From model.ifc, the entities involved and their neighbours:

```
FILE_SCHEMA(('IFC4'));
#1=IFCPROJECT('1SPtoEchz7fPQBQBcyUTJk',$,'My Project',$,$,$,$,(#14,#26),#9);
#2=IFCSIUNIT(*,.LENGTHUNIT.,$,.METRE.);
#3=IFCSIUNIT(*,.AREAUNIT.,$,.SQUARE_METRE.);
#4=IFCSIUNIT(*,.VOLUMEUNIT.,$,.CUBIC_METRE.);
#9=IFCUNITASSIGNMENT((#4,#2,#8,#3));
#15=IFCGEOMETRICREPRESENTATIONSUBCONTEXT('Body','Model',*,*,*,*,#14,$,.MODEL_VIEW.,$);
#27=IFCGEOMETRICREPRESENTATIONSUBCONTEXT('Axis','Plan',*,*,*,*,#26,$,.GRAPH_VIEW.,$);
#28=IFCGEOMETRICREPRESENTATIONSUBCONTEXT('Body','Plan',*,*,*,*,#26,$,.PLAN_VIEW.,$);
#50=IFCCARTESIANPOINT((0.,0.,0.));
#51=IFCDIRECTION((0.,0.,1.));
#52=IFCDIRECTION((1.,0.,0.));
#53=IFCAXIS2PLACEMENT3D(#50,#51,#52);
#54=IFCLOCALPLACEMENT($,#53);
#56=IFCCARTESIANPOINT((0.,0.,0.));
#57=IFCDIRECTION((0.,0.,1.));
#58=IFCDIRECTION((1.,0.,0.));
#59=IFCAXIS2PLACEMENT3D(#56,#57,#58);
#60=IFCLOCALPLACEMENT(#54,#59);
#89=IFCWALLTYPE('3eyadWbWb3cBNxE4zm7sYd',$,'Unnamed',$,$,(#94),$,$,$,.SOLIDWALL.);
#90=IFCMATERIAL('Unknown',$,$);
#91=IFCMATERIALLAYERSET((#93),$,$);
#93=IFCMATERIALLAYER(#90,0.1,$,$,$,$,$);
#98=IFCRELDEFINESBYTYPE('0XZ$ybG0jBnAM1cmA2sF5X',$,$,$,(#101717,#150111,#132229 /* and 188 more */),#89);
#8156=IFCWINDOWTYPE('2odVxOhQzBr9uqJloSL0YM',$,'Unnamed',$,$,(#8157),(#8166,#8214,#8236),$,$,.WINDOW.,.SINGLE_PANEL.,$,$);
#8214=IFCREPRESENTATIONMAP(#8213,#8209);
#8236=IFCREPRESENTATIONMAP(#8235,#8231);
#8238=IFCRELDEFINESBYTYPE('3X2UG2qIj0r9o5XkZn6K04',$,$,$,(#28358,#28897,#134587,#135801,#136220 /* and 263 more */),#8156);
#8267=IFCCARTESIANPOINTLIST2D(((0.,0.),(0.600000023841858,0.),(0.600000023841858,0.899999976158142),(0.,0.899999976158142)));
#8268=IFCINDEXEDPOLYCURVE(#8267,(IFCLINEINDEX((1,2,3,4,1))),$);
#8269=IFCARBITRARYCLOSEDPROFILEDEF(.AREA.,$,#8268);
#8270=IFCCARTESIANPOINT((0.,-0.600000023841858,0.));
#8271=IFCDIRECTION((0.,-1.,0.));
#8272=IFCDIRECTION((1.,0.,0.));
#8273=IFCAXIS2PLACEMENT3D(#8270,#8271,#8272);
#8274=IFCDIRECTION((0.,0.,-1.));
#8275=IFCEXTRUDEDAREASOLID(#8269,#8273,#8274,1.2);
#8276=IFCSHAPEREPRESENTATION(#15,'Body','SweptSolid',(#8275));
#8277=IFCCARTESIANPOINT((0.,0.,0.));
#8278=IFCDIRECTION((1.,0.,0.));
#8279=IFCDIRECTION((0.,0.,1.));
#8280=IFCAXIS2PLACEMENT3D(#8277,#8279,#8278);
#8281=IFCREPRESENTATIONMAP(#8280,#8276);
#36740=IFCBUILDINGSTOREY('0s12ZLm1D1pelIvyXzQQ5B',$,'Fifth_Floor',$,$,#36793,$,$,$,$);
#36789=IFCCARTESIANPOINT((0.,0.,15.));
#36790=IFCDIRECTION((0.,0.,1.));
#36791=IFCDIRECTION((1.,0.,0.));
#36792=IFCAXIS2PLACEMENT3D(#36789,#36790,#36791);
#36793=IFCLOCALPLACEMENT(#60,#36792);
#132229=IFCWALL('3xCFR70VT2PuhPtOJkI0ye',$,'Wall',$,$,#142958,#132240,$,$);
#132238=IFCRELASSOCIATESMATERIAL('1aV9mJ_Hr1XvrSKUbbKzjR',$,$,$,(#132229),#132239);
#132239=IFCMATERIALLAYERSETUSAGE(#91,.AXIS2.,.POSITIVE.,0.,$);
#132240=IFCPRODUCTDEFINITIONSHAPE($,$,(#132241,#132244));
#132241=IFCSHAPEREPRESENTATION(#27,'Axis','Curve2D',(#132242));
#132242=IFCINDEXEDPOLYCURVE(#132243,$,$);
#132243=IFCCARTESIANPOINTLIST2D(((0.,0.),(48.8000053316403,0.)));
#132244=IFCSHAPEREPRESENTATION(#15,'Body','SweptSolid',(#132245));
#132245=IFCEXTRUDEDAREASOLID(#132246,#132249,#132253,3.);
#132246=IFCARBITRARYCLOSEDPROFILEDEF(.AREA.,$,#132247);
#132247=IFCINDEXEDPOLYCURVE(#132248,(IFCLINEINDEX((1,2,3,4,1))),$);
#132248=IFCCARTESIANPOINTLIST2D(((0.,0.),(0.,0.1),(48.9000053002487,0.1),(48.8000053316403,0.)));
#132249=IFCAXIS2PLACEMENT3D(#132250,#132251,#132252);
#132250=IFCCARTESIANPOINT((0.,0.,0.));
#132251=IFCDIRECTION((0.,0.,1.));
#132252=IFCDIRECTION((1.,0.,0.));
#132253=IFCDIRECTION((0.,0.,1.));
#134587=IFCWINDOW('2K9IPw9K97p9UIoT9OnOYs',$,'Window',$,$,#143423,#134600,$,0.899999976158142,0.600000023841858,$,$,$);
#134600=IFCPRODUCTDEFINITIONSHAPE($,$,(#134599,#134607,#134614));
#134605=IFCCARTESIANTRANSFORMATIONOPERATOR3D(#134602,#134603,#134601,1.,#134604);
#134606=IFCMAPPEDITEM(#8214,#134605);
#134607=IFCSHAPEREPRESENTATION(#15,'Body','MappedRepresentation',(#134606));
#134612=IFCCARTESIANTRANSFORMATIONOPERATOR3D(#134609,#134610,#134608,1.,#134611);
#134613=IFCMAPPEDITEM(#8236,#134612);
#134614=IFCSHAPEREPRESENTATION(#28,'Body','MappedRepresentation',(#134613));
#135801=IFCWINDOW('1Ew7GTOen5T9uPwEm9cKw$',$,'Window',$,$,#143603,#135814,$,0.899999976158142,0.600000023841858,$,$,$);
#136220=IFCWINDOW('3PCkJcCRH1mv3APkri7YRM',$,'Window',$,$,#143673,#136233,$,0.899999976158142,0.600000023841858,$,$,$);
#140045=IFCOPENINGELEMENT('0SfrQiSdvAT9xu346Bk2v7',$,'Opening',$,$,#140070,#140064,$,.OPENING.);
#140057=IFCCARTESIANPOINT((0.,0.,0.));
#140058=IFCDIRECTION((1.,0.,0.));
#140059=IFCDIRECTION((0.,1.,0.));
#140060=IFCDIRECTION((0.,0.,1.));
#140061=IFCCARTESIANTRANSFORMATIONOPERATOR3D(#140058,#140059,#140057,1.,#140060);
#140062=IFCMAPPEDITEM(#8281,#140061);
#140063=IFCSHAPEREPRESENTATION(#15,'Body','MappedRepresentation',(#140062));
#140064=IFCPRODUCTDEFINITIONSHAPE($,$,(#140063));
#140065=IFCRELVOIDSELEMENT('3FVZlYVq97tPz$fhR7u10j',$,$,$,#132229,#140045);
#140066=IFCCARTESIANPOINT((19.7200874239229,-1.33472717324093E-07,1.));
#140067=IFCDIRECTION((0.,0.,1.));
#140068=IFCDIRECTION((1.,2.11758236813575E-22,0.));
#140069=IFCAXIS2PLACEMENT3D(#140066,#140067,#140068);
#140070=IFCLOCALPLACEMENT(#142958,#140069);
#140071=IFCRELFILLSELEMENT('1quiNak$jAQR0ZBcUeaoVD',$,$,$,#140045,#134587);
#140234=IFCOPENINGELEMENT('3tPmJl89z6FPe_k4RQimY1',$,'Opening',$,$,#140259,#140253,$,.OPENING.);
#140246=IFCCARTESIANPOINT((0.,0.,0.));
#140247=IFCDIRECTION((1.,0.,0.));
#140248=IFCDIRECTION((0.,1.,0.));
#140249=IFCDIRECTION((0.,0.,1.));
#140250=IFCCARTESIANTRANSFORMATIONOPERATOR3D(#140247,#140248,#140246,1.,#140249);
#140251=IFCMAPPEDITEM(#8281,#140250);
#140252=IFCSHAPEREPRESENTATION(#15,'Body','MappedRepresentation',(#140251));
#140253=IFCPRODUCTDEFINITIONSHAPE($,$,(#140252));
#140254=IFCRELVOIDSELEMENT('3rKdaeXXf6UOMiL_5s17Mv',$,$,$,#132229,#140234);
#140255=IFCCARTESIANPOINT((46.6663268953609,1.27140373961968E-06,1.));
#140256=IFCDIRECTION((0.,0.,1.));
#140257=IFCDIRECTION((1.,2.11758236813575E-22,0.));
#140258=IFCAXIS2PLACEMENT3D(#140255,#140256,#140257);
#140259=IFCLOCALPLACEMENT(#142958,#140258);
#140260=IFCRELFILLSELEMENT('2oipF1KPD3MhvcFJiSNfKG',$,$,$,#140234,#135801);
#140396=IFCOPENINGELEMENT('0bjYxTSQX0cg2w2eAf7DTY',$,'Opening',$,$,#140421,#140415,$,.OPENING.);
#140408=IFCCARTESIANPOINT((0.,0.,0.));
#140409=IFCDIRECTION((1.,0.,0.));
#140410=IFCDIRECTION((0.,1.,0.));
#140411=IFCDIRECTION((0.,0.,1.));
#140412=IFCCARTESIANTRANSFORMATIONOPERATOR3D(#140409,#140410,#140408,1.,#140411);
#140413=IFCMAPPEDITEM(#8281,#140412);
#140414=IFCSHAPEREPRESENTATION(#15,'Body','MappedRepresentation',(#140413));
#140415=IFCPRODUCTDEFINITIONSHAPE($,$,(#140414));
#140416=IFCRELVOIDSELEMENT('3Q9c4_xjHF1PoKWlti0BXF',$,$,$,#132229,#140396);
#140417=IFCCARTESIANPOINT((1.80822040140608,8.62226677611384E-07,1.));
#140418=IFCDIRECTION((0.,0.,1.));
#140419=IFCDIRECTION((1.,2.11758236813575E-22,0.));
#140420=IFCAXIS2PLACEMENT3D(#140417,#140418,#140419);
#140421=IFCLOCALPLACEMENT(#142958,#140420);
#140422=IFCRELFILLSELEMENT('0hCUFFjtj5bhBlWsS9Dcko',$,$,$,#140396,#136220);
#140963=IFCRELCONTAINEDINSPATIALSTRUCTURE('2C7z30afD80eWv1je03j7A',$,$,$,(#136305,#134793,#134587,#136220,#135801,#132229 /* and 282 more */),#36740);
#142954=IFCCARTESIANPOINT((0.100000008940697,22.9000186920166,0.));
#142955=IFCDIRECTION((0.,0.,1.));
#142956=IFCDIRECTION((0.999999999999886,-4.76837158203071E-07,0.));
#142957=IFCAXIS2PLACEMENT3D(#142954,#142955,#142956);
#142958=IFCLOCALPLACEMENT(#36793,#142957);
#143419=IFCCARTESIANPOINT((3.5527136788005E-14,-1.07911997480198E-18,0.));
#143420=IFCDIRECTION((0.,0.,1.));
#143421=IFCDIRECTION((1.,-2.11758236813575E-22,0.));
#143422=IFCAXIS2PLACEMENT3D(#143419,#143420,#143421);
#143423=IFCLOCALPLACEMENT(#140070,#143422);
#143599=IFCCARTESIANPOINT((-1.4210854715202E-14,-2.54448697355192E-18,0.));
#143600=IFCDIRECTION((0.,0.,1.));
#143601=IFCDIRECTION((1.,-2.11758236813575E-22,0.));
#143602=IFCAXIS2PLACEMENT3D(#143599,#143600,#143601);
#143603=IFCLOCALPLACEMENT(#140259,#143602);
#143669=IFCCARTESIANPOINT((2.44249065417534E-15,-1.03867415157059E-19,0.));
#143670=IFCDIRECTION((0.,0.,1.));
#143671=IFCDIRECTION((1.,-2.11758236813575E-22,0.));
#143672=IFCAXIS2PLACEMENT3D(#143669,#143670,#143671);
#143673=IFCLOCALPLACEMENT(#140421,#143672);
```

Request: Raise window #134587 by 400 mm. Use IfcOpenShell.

```python
import numpy as np
import ifcopenshell
import ifcopenshell.api.geometry
import ifcopenshell.util.placement
import ifcopenshell.util.unit

model = ifcopenshell.open("model.ifc")
unit_scale = ifcopenshell.util.unit.calculate_unit_scale(model)

window = model.by_guid("2K9IPw9K97p9UIoT9OnOYs")
opening = window.FillsVoids[0].RelatingOpeningElement
dz = 0.4 / unit_scale

shift = np.array([0.0, 0.0, dz])
# The window is placed relative to its opening, so it follows when the opening moves.
matrix = ifcopenshell.util.placement.get_local_placement(opening.ObjectPlacement)
matrix[:3, 3] += shift
ifcopenshell.api.geometry.edit_object_placement(
    model, product=opening, matrix=matrix, is_si=False, should_transform_children=True
)

print(f"moved by {dz * unit_scale:+.3f} m")

model.write("model_edited.ifc")
```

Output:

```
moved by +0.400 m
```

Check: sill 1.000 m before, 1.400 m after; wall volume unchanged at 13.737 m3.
